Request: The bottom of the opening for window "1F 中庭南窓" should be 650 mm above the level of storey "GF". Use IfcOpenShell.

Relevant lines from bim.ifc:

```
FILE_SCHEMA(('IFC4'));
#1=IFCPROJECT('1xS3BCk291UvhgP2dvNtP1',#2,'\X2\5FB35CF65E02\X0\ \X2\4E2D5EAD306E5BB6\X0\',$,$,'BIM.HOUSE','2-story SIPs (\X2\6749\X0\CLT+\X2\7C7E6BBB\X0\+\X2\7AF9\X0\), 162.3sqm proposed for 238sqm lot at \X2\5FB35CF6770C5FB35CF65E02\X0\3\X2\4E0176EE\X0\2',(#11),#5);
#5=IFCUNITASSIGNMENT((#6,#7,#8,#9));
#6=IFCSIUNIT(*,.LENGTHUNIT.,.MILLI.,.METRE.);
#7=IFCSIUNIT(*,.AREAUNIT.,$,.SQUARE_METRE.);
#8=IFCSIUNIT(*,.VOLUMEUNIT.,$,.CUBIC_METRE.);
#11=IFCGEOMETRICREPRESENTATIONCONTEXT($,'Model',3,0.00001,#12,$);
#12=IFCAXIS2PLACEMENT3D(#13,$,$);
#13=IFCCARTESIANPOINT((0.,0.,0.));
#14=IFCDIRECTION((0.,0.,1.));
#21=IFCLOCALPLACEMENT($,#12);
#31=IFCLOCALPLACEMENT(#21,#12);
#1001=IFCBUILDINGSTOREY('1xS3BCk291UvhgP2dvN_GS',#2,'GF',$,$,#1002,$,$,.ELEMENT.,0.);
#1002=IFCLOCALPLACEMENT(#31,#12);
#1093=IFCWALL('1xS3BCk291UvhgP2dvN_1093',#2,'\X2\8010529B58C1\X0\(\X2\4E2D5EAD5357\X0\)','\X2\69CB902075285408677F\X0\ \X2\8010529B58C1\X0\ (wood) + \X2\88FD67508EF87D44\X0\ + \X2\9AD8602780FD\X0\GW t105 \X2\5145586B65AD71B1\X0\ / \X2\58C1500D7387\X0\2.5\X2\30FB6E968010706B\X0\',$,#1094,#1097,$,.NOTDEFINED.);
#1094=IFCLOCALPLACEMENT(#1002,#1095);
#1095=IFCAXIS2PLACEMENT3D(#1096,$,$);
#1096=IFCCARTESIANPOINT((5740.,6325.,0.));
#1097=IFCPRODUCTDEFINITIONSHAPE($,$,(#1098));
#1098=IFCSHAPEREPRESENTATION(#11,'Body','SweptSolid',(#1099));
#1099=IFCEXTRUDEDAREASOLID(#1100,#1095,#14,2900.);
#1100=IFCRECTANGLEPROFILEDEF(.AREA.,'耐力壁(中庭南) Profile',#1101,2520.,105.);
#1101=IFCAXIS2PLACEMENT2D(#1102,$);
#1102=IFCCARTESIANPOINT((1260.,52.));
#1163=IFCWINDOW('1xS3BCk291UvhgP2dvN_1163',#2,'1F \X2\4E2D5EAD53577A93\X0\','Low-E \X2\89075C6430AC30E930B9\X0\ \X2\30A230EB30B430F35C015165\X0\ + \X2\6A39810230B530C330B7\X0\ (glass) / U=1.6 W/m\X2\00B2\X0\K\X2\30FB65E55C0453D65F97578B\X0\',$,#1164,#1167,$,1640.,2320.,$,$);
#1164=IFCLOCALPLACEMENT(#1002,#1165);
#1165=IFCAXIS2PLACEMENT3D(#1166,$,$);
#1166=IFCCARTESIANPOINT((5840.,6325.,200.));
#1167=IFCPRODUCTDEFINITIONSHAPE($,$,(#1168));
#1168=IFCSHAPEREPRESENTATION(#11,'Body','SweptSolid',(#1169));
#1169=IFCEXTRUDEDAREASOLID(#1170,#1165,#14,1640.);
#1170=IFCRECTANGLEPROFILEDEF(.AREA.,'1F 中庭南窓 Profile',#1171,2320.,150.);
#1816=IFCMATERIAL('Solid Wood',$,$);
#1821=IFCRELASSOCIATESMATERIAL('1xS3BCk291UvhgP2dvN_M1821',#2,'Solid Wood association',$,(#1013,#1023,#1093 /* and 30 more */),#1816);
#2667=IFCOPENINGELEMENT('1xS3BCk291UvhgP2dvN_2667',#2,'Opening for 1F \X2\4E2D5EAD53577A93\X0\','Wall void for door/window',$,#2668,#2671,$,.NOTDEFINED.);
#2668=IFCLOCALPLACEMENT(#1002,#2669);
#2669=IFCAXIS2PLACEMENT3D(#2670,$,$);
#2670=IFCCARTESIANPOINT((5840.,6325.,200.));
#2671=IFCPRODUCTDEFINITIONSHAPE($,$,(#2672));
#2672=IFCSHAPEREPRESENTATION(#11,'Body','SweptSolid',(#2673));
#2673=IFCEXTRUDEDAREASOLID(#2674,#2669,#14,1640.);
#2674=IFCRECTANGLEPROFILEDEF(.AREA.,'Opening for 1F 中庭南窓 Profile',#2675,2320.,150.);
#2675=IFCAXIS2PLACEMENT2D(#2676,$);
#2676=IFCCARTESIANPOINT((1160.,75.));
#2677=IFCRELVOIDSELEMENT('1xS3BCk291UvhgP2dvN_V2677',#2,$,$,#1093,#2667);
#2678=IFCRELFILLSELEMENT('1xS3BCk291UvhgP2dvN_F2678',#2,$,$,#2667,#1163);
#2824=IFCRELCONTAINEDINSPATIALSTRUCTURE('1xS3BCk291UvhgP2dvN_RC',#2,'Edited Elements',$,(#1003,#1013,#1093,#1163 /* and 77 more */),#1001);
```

```python
import numpy as np
import ifcopenshell
import ifcopenshell.api.geometry
import ifcopenshell.geom
import ifcopenshell.util.element
import ifcopenshell.util.placement
import ifcopenshell.util.shape
import ifcopenshell.util.unit

model = ifcopenshell.open("bim.ifc")
unit_scale = ifcopenshell.util.unit.calculate_unit_scale(model)

window = model.by_guid("1xS3BCk291UvhgP2dvN_1163")
opening = window.FillsVoids[0].RelatingOpeningElement
storey = ifcopenshell.util.element.get_container(window, ifc_class="IfcBuildingStorey")
level = ifcopenshell.util.placement.get_local_placement(storey.ObjectPlacement)[2, 3]

# The opening's origin need not be at the sill, so measure its lowest point.
shape = ifcopenshell.geom.create_shape(ifcopenshell.geom.settings(), opening)
bottom = ifcopenshell.util.shape.get_shape_bottom_elevation(shape, shape.geometry) / unit_scale
dz = level + 0.65 / unit_scale - bottom

shift = np.array([0.0, 0.0, dz])
# The window is not placed relative to its opening, so move both.
for product in (opening, window):
    matrix = ifcopenshell.util.placement.get_local_placement(product.ObjectPlacement)
    matrix[:3, 3] += shift
    ifcopenshell.api.geometry.edit_object_placement(model, product=product, matrix=matrix, is_si=False)

print(f"moved by {dz * unit_scale:+.3f} m")

model.write("bim_updated.ifc")
```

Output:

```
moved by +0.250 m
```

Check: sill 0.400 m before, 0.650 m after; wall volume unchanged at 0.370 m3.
